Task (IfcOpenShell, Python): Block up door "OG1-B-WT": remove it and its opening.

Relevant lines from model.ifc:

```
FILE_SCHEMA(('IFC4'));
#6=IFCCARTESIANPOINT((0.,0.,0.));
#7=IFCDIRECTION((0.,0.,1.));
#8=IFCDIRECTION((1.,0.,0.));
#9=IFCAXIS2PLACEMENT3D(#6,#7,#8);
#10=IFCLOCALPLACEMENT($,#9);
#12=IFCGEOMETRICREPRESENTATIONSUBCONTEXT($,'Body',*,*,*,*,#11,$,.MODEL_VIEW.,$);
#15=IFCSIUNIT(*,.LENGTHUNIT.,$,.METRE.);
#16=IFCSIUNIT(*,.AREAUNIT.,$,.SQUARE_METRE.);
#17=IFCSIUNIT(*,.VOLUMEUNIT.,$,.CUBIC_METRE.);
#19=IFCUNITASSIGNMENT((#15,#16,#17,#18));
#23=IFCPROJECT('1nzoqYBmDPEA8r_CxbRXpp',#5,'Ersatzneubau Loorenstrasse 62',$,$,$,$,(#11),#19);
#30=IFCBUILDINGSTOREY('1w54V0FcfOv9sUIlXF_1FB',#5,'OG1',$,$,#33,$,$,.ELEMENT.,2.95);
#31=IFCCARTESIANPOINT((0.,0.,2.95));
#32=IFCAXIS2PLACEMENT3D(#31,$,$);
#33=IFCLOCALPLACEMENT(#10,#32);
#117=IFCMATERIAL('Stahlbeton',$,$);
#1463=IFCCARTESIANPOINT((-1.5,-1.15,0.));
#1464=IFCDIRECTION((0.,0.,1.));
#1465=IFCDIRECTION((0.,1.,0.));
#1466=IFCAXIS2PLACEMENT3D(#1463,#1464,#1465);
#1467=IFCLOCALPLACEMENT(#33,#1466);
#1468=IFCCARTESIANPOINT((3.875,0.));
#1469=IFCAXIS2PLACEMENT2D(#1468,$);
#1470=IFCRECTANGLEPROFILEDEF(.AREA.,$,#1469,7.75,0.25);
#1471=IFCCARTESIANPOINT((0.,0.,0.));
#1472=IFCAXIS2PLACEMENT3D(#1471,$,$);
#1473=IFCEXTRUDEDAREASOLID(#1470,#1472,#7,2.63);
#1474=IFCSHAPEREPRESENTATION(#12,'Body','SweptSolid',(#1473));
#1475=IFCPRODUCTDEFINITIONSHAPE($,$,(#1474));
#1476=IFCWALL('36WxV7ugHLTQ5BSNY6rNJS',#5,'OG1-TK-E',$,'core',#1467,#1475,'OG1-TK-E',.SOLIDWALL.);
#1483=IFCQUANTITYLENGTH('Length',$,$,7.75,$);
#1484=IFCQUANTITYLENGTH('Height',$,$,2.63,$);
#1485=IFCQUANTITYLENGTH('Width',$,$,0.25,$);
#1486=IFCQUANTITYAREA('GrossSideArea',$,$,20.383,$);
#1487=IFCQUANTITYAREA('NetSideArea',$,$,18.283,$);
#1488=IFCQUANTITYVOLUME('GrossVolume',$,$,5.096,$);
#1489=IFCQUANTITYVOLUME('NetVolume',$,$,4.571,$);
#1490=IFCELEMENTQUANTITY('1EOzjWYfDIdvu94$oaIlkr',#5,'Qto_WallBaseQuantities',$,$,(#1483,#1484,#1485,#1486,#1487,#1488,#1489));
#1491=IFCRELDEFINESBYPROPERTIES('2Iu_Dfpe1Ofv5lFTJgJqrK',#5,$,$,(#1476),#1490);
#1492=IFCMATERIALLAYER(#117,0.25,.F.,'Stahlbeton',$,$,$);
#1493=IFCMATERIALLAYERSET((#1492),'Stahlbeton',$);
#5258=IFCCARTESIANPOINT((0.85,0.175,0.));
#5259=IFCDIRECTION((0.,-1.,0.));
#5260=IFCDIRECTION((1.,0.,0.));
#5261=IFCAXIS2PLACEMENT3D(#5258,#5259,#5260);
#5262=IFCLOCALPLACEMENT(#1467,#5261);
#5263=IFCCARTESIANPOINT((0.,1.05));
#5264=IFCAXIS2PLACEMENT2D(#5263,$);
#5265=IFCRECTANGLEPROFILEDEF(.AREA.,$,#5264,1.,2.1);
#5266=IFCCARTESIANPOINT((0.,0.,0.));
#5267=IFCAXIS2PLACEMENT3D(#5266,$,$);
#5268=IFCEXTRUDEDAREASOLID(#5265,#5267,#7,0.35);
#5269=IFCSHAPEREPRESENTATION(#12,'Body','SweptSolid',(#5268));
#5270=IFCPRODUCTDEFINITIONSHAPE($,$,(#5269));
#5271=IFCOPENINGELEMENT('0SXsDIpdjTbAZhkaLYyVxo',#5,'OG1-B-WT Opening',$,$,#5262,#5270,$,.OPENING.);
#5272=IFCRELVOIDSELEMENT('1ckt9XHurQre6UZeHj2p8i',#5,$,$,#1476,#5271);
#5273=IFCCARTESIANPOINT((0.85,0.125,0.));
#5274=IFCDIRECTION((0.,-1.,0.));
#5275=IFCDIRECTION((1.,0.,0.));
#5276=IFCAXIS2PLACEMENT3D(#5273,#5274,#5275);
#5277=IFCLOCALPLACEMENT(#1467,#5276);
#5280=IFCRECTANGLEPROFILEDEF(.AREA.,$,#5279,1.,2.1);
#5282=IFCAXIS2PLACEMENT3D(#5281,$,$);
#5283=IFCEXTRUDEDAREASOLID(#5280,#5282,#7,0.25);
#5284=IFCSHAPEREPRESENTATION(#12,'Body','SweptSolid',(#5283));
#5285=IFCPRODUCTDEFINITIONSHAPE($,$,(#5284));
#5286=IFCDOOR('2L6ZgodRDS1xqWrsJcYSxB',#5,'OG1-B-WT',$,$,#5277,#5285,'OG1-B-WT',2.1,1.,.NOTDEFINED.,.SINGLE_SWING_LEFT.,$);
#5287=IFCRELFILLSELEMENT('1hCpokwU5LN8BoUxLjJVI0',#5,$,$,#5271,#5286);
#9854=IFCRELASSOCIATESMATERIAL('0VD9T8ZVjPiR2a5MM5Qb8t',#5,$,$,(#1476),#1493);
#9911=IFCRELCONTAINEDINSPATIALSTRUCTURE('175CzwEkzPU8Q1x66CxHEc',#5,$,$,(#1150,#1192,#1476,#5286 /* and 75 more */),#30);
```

```python
import ifcopenshell
import ifcopenshell.api.feature
import ifcopenshell.api.pset
import ifcopenshell.api.root
import ifcopenshell.geom
import ifcopenshell.util.element
import ifcopenshell.util.shape
import ifcopenshell.util.unit

model = ifcopenshell.open("model.ifc")
area_scale = ifcopenshell.util.unit.calculate_unit_scale(model, "AREAUNIT")
volume_scale = ifcopenshell.util.unit.calculate_unit_scale(model, "VOLUMEUNIT")
settings = ifcopenshell.geom.settings()


def volume(element):
    """Net volume in cubic metres, openings subtracted."""
    shape = ifcopenshell.geom.create_shape(settings, element)
    return ifcopenshell.util.shape.get_volume(shape.geometry)


door = model.by_guid("2L6ZgodRDS1xqWrsJcYSxB")
opening = door.FillsVoids[0].RelatingOpeningElement
wall = opening.VoidsElements[0].RelatingBuildingElement
before = volume(wall)

ifcopenshell.api.root.remove_product(model, product=door)
ifcopenshell.api.feature.remove_feature(model, feature=opening)

after = volume(wall)
thickness = 0.25  # wall thickness in metres

# Update the wall's stored quantities.
qto = model.by_id(ifcopenshell.util.element.get_pset(wall, "Qto_WallBaseQuantities", should_inherit=False)["id"])
ifcopenshell.api.pset.edit_qto(model, qto=qto, properties={
    "NetSideArea": after / thickness / area_scale,
    "NetVolume": after / volume_scale,
})

print(f"wall volume {before:.3f} -> {after:.3f} m3")

model.write("model_edited.ifc")
```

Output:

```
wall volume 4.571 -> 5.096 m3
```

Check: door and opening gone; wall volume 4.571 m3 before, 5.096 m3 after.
